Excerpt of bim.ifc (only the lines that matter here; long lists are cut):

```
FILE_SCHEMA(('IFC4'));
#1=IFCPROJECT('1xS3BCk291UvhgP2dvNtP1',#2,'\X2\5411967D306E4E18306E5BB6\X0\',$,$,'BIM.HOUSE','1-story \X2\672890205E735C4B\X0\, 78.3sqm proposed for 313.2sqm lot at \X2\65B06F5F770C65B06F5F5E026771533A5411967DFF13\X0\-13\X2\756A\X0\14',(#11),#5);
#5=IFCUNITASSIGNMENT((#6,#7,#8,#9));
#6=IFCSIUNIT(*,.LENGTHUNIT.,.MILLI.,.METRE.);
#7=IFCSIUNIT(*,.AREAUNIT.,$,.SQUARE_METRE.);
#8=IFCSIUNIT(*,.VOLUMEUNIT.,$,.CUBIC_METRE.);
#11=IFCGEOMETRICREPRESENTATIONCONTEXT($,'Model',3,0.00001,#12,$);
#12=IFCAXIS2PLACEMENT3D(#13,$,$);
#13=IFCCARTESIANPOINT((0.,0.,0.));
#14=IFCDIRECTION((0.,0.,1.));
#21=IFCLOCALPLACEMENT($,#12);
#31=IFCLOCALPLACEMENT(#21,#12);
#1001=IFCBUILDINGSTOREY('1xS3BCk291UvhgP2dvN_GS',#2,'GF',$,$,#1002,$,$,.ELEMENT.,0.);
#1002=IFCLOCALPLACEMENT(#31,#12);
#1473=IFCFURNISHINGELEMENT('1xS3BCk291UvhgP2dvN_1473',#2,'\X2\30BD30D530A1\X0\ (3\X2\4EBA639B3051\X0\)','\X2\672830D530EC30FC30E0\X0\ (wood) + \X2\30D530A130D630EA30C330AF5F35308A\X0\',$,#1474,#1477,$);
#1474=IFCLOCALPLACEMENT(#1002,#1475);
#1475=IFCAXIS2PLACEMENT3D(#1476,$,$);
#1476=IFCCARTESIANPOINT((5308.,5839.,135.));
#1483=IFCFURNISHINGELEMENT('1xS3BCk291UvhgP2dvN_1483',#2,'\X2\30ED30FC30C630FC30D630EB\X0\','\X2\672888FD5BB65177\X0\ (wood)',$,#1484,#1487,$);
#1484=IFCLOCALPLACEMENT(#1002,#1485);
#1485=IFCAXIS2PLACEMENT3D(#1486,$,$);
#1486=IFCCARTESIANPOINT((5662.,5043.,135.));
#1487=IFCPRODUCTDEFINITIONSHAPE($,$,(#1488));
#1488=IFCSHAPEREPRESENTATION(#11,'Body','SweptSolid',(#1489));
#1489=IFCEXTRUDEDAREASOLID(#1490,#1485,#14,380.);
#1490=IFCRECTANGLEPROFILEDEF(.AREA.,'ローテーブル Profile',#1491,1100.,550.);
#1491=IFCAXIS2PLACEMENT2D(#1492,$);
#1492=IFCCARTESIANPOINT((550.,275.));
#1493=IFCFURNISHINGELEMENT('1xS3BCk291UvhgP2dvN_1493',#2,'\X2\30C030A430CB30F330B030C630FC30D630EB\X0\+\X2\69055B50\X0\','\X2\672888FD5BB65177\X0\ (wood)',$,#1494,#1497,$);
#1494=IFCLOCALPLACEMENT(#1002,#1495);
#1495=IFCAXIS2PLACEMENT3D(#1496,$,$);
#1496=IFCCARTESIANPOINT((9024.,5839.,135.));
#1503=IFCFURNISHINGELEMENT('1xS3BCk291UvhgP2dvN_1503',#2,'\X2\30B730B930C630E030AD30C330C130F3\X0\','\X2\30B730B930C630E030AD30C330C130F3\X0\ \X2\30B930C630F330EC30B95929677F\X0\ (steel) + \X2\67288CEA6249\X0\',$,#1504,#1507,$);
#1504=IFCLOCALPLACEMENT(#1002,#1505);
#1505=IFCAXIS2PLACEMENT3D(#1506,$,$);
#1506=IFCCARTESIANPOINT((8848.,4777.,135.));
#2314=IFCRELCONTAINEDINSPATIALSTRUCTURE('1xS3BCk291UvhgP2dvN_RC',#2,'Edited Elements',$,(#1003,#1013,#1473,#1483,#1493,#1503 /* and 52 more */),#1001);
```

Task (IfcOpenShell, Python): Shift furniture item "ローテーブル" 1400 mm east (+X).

```python
import ifcopenshell
import ifcopenshell.api.geometry
import ifcopenshell.util.placement
import ifcopenshell.util.unit

model = ifcopenshell.open("bim.ifc")
unit_scale = ifcopenshell.util.unit.calculate_unit_scale(model)

item = model.by_id(1483)
matrix = ifcopenshell.util.placement.get_local_placement(item.ObjectPlacement)
matrix[0, 3] += 1.4 / unit_scale
ifcopenshell.api.geometry.edit_object_placement(model, product=item, matrix=matrix, is_si=False)

print(ifcopenshell.util.placement.get_local_placement(item.ObjectPlacement).round(3) + 0.0)

model.write("bim_rev.ifc")
```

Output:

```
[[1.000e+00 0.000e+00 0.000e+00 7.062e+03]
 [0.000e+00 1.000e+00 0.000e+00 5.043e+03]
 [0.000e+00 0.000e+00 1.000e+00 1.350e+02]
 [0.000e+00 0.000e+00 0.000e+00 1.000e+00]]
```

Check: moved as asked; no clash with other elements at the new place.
